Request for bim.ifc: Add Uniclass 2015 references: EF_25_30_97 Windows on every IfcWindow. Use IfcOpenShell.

First a look at what the model holds.

```python
import ifcopenshell

model = ifcopenshell.open("bim.ifc")
print(model.schema)
print("classifications:", [c.Name for c in model.by_type("IfcClassification")])
for ifc_class in ("IfcDoor", "IfcRoof", "IfcStair", "IfcWall", "IfcWindow"):
    print(ifc_class, len(model.by_type(ifc_class)))
```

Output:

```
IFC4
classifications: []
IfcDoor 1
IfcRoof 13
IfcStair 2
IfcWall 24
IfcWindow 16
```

```python
import ifcopenshell
import ifcopenshell.api.classification

model = ifcopenshell.open("bim.ifc")

system = ifcopenshell.api.classification.add_classification(model, classification="Uniclass 2015")

codes = {
    "IfcWindow": ("EF_25_30_97", "Windows"),
}
for ifc_class, (code, name) in codes.items():
    products = model.by_type(ifc_class)
    ifcopenshell.api.classification.add_reference(
        model, products=products, classification=system, identification=code, name=name
    )
    print(code, len(products))

model.write("bim_updated.ifc")
```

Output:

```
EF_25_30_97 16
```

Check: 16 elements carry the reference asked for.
